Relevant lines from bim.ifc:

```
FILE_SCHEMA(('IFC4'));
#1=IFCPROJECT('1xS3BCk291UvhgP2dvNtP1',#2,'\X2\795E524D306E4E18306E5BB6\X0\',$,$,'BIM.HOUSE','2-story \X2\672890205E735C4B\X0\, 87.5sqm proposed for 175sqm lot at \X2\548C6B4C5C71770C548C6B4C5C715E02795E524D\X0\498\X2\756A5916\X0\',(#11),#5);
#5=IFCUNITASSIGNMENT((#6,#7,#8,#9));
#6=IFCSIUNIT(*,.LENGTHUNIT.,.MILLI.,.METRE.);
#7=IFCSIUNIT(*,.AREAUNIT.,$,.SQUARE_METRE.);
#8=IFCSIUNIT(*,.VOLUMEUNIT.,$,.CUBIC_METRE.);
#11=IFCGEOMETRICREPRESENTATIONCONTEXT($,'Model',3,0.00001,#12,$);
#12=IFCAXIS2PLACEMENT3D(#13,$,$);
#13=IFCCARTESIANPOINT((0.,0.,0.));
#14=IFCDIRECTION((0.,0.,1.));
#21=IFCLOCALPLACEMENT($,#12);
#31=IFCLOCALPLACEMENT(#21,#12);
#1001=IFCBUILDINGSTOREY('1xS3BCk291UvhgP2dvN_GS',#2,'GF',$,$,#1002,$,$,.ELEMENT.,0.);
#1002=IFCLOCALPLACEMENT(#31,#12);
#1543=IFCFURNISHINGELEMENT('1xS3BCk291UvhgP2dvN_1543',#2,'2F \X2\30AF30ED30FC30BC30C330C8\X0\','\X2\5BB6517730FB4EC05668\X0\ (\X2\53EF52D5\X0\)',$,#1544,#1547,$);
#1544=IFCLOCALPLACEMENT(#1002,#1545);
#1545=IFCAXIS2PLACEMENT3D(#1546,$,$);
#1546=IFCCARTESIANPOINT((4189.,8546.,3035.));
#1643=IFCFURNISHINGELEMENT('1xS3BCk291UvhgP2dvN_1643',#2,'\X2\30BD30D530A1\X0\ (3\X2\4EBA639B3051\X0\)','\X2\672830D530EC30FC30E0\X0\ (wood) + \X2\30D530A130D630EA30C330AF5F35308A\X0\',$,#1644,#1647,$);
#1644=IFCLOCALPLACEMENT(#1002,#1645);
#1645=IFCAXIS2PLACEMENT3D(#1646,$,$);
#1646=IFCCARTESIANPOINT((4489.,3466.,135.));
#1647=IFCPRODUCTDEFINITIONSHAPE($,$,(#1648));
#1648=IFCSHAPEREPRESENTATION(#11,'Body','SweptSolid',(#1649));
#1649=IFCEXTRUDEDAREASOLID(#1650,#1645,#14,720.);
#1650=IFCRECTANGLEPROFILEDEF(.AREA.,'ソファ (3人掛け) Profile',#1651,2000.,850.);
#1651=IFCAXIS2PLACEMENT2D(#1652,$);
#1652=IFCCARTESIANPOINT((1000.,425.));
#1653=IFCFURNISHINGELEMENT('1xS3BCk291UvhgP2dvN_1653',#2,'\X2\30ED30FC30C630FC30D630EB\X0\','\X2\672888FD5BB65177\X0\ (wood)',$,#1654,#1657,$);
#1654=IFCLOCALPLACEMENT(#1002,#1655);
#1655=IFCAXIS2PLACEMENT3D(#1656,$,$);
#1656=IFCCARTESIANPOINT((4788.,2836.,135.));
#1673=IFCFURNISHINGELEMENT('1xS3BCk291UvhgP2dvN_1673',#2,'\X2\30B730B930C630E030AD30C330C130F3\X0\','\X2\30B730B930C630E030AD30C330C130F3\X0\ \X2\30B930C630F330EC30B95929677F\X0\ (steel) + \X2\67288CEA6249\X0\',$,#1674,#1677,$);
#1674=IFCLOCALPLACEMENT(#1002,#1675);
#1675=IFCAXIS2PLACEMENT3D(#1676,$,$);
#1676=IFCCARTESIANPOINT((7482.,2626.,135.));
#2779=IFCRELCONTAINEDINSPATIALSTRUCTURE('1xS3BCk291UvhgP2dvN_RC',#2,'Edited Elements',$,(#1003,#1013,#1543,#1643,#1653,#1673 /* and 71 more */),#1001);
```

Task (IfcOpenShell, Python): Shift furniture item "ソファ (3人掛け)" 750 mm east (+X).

```python
import ifcopenshell
import ifcopenshell.api.geometry
import ifcopenshell.util.placement
import ifcopenshell.util.unit

model = ifcopenshell.open("bim.ifc")
unit_scale = ifcopenshell.util.unit.calculate_unit_scale(model)

item = model.by_guid("1xS3BCk291UvhgP2dvN_1643")
matrix = ifcopenshell.util.placement.get_local_placement(item.ObjectPlacement)
matrix[0, 3] += 0.75 / unit_scale
ifcopenshell.api.geometry.edit_object_placement(model, product=item, matrix=matrix, is_si=False)

print(ifcopenshell.util.placement.get_local_placement(item.ObjectPlacement).round(3) + 0.0)

model.write("bim-out.ifc")
```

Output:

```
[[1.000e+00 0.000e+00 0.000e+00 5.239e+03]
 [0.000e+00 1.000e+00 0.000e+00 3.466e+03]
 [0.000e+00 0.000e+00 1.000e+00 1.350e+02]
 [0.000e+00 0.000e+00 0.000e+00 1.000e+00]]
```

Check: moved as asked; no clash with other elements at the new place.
